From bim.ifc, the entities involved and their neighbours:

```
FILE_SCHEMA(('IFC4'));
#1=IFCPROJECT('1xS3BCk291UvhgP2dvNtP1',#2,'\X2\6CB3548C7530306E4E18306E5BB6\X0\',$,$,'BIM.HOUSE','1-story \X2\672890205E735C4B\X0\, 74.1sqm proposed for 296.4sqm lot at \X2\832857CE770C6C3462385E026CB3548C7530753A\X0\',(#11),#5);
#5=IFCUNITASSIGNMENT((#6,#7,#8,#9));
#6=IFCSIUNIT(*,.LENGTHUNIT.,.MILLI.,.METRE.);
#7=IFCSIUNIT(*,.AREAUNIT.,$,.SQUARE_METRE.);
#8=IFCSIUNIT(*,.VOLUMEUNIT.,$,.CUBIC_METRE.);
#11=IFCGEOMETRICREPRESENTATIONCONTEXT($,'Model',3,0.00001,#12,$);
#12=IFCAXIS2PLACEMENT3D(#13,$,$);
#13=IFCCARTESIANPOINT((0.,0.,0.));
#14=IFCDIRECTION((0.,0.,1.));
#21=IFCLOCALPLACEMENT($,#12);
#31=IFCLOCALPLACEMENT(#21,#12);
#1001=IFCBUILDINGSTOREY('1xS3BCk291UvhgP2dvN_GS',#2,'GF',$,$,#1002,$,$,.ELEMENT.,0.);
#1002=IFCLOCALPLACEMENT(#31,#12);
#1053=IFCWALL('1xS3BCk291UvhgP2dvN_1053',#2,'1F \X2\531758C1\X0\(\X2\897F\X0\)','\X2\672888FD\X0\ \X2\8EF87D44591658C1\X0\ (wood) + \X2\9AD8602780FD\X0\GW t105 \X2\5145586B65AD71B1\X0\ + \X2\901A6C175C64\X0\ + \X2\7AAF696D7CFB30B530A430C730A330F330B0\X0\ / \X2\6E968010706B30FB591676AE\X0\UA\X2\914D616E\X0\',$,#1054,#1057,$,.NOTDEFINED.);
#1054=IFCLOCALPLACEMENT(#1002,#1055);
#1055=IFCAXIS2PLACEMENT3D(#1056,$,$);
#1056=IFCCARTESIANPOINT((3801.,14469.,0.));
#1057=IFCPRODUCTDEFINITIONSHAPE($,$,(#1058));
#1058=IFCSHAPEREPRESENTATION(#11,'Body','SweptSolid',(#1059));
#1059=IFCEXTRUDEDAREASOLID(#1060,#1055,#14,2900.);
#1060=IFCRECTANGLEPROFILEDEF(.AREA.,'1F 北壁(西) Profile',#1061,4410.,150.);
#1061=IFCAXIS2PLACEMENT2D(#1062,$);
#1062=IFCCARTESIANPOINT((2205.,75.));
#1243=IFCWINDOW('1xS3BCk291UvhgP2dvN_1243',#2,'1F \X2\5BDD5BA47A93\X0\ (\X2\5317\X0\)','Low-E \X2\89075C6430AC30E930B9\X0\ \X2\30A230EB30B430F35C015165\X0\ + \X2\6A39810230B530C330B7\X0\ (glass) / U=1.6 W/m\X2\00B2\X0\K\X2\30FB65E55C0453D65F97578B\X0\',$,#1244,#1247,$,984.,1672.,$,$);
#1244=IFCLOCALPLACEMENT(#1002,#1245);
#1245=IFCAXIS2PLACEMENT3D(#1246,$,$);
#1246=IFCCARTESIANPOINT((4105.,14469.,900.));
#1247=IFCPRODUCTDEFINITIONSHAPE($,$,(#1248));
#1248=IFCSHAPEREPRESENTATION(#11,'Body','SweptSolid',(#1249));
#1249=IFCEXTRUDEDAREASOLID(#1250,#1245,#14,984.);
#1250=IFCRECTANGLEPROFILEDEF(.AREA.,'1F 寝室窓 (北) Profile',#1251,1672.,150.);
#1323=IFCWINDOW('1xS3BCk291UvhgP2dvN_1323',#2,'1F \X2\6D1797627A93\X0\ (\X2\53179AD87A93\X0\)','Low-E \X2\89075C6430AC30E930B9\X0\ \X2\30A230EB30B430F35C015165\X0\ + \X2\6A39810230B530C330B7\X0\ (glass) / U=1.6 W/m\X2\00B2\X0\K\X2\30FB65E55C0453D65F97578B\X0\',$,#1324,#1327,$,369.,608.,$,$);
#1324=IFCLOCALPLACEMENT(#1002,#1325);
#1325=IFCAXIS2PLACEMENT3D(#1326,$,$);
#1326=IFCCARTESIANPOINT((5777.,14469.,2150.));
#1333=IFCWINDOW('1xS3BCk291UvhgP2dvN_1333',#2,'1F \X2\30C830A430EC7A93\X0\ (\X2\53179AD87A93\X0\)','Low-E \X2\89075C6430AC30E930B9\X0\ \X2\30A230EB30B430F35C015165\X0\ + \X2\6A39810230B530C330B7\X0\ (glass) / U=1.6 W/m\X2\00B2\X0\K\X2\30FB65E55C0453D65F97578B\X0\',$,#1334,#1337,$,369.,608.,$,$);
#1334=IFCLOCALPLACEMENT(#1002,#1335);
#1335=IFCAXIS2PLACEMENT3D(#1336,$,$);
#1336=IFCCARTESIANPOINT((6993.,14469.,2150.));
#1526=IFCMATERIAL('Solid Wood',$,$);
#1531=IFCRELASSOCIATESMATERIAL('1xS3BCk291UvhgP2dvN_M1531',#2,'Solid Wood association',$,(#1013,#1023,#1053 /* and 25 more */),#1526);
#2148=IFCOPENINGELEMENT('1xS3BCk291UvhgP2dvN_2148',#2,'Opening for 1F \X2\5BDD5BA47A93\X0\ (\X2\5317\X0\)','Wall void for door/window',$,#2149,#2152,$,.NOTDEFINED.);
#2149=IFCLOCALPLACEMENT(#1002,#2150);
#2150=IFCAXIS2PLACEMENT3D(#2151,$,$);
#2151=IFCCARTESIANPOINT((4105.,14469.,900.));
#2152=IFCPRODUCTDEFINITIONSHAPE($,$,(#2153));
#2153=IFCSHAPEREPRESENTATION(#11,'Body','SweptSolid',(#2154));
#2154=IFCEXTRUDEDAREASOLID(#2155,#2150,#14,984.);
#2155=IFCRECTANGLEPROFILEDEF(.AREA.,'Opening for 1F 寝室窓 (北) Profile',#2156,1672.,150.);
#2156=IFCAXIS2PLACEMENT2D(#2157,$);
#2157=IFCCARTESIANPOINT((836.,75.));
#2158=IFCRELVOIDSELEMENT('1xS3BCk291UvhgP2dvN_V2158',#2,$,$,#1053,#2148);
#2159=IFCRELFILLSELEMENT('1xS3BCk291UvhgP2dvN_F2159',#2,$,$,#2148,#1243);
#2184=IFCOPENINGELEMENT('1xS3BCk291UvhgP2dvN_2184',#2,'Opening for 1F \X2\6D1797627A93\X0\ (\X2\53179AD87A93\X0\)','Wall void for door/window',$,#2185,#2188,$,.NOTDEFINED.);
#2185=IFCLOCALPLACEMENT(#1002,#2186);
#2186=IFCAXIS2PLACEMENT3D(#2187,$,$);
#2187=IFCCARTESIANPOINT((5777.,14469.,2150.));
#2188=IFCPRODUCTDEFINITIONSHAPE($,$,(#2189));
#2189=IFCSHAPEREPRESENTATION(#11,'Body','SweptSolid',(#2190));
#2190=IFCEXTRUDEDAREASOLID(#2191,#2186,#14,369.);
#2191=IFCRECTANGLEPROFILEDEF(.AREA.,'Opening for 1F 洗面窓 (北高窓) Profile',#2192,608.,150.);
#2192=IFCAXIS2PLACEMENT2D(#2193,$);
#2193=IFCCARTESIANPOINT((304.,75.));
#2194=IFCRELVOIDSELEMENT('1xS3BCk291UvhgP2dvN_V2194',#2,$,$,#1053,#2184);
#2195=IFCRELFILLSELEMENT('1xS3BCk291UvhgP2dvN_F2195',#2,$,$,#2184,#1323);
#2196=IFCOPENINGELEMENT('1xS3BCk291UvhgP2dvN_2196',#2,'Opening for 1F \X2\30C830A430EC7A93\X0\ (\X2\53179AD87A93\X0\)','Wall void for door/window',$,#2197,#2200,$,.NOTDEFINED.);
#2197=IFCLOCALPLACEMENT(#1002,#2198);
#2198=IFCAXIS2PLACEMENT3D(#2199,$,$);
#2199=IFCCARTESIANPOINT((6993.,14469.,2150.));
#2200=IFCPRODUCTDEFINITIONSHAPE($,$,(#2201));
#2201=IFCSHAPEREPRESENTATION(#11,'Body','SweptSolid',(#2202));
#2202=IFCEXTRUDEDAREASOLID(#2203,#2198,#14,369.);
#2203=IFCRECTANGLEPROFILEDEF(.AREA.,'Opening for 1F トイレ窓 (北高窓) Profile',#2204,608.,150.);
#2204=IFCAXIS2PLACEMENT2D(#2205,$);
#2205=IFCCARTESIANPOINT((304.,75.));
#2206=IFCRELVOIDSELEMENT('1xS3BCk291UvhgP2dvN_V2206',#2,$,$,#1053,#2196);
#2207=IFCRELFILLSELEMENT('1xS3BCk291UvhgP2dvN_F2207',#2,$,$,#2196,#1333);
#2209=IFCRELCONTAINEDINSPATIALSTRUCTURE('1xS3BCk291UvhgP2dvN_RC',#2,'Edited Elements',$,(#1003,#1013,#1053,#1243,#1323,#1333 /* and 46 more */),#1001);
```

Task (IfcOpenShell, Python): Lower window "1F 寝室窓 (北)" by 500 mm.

```python
import numpy as np
import ifcopenshell
import ifcopenshell.api.geometry
import ifcopenshell.util.placement
import ifcopenshell.util.unit

model = ifcopenshell.open("bim.ifc")
unit_scale = ifcopenshell.util.unit.calculate_unit_scale(model)

window = model.by_id(1243)
opening = window.FillsVoids[0].RelatingOpeningElement
dz = -0.5 / unit_scale

shift = np.array([0.0, 0.0, dz])
# The window is not placed relative to its opening, so move both.
for product in (opening, window):
    matrix = ifcopenshell.util.placement.get_local_placement(product.ObjectPlacement)
    matrix[:3, 3] += shift
    ifcopenshell.api.geometry.edit_object_placement(model, product=product, matrix=matrix, is_si=False)

print(f"moved by {dz * unit_scale:+.3f} m")

model.write("bim-out.ifc")
```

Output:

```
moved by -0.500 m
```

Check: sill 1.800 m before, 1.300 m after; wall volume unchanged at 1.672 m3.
